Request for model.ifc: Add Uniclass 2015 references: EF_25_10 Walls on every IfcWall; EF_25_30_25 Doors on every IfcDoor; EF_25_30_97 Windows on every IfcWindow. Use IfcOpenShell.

First a look at what the model holds.

```python
import ifcopenshell

model = ifcopenshell.open("model.ifc")
print(model.schema)
print("classifications:", [c.Name for c in model.by_type("IfcClassification")])
for ifc_class in ("IfcDoor", "IfcRoof", "IfcStair", "IfcWall", "IfcWindow"):
    print(ifc_class, len(model.by_type(ifc_class)))
```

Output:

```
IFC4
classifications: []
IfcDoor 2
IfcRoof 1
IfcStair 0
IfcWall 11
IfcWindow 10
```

```python
import ifcopenshell
import ifcopenshell.api.classification

model = ifcopenshell.open("model.ifc")

system = ifcopenshell.api.classification.add_classification(model, classification="Uniclass 2015")

codes = {
    "IfcWall": ("EF_25_10", "Walls"),
    "IfcDoor": ("EF_25_30_25", "Doors"),
    "IfcWindow": ("EF_25_30_97", "Windows"),
}
for ifc_class, (code, name) in codes.items():
    products = model.by_type(ifc_class)
    ifcopenshell.api.classification.add_reference(
        model, products=products, classification=system, identification=code, name=name
    )
    print(code, len(products))

model.write("model_updated.ifc")
```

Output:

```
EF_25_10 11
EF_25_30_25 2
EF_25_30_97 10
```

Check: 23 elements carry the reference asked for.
